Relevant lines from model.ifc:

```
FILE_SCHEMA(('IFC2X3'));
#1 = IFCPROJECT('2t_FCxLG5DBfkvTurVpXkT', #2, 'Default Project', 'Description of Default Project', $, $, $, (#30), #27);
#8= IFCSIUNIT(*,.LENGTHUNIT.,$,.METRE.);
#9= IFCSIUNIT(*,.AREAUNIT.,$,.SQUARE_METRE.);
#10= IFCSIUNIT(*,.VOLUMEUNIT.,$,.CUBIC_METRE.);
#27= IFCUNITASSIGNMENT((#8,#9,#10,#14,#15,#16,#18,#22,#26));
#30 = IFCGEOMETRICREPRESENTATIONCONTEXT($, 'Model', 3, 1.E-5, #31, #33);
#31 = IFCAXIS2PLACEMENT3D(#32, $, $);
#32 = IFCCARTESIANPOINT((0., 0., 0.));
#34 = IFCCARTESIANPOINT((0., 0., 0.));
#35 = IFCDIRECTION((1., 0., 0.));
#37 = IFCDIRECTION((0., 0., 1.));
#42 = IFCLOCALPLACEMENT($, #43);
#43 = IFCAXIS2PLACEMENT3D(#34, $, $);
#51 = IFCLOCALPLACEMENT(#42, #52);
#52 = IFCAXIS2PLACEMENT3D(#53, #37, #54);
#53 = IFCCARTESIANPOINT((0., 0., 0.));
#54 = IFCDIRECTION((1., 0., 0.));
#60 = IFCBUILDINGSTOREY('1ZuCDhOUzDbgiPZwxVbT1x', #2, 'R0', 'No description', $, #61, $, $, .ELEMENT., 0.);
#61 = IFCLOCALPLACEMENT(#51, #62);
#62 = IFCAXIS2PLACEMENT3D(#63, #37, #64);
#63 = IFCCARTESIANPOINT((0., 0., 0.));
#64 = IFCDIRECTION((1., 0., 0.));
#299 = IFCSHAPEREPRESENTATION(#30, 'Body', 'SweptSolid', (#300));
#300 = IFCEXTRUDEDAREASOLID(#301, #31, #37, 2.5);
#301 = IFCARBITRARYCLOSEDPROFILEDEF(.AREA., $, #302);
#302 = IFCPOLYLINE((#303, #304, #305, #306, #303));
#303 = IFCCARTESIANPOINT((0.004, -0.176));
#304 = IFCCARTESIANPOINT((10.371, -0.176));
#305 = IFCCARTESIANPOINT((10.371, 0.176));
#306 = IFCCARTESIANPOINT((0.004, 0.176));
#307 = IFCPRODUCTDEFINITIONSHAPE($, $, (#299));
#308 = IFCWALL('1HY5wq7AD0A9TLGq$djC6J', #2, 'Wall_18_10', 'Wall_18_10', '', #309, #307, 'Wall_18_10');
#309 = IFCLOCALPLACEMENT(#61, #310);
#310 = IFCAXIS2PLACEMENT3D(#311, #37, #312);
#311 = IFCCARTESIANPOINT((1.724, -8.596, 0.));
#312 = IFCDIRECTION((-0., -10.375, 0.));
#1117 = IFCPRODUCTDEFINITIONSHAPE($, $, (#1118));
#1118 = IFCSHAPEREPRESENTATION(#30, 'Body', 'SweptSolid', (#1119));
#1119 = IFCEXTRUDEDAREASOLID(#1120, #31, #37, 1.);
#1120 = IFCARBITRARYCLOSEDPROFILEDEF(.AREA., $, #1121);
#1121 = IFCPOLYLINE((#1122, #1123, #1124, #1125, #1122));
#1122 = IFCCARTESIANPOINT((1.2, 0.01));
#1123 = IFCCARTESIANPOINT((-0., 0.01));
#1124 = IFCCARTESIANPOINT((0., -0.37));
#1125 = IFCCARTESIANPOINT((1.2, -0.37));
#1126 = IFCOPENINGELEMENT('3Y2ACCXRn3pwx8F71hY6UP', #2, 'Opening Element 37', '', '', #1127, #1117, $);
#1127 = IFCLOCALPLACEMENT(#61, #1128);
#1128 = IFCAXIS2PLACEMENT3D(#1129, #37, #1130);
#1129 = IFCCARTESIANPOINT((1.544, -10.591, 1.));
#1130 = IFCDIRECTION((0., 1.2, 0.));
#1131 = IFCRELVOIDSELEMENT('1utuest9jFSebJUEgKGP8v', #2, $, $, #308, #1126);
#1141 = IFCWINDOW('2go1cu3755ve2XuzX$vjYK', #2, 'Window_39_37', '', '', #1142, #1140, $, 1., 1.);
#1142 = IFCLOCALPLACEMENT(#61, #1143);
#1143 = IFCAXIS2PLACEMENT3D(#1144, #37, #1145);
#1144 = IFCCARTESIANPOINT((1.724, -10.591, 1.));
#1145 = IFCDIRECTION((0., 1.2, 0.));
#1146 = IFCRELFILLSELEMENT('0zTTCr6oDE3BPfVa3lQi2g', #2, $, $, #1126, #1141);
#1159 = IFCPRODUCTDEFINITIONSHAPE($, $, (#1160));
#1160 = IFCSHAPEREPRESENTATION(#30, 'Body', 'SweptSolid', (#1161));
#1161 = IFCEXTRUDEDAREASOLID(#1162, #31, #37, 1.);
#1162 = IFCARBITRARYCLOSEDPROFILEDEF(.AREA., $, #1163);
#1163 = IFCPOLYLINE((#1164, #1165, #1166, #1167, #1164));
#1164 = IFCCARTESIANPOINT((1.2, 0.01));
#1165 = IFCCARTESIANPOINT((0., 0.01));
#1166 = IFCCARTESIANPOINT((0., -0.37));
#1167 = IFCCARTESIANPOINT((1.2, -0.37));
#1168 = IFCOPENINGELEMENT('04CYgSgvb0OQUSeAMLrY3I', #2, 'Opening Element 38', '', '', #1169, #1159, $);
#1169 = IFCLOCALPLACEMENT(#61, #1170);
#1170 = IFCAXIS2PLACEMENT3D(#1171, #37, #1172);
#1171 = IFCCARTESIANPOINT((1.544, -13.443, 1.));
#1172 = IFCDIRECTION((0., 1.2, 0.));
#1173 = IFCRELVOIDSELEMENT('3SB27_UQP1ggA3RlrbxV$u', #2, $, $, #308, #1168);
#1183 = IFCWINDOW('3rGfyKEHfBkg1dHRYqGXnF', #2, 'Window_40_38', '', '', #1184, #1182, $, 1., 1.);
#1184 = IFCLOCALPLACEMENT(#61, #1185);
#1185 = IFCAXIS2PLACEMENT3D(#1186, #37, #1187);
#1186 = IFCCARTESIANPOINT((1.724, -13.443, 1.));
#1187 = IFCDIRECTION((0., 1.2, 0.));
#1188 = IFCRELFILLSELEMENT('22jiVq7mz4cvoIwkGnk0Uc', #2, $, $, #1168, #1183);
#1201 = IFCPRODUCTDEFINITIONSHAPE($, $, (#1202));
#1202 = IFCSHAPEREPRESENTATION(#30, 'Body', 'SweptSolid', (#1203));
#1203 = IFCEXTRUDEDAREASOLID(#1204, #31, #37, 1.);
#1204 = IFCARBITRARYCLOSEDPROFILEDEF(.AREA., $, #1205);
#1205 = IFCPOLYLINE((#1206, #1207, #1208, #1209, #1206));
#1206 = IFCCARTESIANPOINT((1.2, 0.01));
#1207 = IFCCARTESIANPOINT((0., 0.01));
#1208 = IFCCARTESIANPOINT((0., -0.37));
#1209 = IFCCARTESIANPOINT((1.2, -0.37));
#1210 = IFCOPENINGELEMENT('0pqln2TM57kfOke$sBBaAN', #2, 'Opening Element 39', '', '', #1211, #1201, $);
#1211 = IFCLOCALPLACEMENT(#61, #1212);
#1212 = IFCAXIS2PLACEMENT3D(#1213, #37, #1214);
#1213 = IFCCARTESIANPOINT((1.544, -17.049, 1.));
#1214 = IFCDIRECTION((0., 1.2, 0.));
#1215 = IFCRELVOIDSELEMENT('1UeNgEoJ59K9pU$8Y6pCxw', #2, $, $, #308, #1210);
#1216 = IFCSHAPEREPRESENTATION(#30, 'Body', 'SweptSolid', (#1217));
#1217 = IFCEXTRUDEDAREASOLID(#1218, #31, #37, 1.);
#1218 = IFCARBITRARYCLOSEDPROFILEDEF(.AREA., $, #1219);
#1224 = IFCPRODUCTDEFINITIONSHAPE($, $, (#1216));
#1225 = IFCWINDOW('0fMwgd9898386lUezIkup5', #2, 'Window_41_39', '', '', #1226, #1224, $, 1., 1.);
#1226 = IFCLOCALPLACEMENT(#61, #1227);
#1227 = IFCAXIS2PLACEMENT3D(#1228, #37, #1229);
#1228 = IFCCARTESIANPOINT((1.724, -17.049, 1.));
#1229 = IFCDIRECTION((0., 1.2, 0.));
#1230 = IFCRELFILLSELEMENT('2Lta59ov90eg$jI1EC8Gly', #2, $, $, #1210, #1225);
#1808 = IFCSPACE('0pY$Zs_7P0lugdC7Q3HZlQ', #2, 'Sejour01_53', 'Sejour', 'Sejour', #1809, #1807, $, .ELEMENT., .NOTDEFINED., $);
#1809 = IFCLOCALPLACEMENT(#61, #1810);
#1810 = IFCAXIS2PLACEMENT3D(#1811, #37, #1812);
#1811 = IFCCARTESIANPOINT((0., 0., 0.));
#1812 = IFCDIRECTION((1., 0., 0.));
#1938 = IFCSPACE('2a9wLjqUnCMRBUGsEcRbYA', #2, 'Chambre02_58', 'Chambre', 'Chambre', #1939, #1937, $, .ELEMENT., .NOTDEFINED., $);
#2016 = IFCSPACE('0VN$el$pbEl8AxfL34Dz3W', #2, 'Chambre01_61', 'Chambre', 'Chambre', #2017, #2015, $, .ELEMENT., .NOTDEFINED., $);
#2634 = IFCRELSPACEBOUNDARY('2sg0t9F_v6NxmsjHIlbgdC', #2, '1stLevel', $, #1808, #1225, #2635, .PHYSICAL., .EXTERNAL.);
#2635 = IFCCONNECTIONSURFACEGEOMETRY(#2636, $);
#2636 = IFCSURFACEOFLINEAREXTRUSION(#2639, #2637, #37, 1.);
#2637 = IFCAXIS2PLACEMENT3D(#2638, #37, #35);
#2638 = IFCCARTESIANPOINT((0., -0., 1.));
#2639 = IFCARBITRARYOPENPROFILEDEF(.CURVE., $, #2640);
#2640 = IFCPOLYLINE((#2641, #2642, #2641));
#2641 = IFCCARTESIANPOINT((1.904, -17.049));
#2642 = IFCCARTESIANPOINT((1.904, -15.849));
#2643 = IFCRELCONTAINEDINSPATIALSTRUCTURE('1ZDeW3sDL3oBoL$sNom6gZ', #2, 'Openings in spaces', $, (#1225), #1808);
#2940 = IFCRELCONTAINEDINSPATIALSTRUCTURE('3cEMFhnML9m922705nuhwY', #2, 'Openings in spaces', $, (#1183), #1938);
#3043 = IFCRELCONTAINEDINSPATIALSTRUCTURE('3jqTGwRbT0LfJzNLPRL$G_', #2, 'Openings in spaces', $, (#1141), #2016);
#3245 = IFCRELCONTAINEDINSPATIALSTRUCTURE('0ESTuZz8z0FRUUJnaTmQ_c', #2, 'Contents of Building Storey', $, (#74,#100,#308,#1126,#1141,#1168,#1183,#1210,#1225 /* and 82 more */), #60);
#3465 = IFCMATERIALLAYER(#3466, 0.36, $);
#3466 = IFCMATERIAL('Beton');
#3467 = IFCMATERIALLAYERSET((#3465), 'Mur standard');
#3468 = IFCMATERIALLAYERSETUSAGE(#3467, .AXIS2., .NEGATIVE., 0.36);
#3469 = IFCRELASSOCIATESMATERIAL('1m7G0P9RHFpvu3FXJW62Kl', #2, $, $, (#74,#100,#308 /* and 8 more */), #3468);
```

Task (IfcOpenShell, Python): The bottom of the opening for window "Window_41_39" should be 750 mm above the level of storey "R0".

```python
import numpy as np
import ifcopenshell
import ifcopenshell.api.geometry
import ifcopenshell.geom
import ifcopenshell.util.element
import ifcopenshell.util.placement
import ifcopenshell.util.shape
import ifcopenshell.util.unit

model = ifcopenshell.open("model.ifc")
unit_scale = ifcopenshell.util.unit.calculate_unit_scale(model)

window = model.by_guid("0fMwgd9898386lUezIkup5")
opening = window.FillsVoids[0].RelatingOpeningElement
storey = ifcopenshell.util.element.get_container(window, ifc_class="IfcBuildingStorey")
level = ifcopenshell.util.placement.get_local_placement(storey.ObjectPlacement)[2, 3]

# The opening's origin need not be at the sill, so measure its lowest point.
shape = ifcopenshell.geom.create_shape(ifcopenshell.geom.settings(), opening)
bottom = ifcopenshell.util.shape.get_shape_bottom_elevation(shape, shape.geometry) / unit_scale
dz = level + 0.75 / unit_scale - bottom

shift = np.array([0.0, 0.0, dz])
# The window is not placed relative to its opening, so move both.
for product in (opening, window):
    matrix = ifcopenshell.util.placement.get_local_placement(product.ObjectPlacement)
    matrix[:3, 3] += shift
    ifcopenshell.api.geometry.edit_object_placement(model, product=product, matrix=matrix, is_si=False)

# Space boundary surfaces are stored in each space's coordinates; move them too.
for rel in window.ProvidesBoundaries:
    if not rel.ConnectionGeometry:
        continue
    surface = rel.ConnectionGeometry.SurfaceOnRelatingElement
    space_matrix = ifcopenshell.util.placement.get_local_placement(rel.RelatingSpace.ObjectPlacement)
    point = np.array(surface.Position.Location.Coordinates) + space_matrix[:3, :3].T @ shift
    surface.Position = model.createIfcAxis2Placement3D(
        model.createIfcCartesianPoint(point.tolist()), surface.Position.Axis, surface.Position.RefDirection
    )

print(f"moved by {dz * unit_scale:+.3f} m")

model.write("model_updated.ifc")
```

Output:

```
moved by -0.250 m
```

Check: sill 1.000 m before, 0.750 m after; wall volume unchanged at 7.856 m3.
